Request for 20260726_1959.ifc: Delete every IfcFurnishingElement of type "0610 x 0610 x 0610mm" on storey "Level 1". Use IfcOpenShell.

First a look at what the model holds.

```python
import ifcopenshell
import ifcopenshell.util.element

model = ifcopenshell.open("20260726_1959.ifc")
print(model.schema)
storey = next(s for s in model.by_type("IfcBuildingStorey") if s.Name == "Level 1")
furniture = [e for e in ifcopenshell.util.element.get_decomposition(storey) if e.is_a("IfcFurnishingElement")]
seen = {}
for e in furniture:
    element_type = ifcopenshell.util.element.get_type(e)
    name = element_type.Name if element_type not in (None, e) else None
    seen[name] = seen.get(name, 0) + 1
for name, count in sorted(seen.items(), key=str):
    print(count, "x", name)
```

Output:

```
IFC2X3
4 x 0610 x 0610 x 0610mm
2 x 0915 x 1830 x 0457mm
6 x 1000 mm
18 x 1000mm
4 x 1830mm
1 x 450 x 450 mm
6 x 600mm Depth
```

```python
import ifcopenshell
import ifcopenshell.api.root
import ifcopenshell.util.element

model = ifcopenshell.open("20260726_1959.ifc")

storey = next(s for s in model.by_type("IfcBuildingStorey") if s.Name == "Level 1")
furniture = [e for e in ifcopenshell.util.element.get_decomposition(storey) if e.is_a("IfcFurnishingElement")]
targets = [e for e in furniture if (t := ifcopenshell.util.element.get_type(e)) not in (None, e) and t.Name == "0610 x 0610 x 0610mm"]

for e in targets:
    ifcopenshell.api.root.remove_product(model, product=e)
print(len(targets), "removed")

model.write("20260726_1959-out.ifc")
```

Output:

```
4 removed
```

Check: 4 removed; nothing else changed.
